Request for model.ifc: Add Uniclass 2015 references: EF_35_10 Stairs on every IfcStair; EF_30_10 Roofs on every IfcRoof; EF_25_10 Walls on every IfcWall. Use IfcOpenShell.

First a look at what the model holds.

```python
import ifcopenshell

model = ifcopenshell.open("model.ifc")
print(model.schema)
print("classifications:", [c.Name for c in model.by_type("IfcClassification")])
for ifc_class in ("IfcDoor", "IfcRoof", "IfcStair", "IfcWall", "IfcWindow"):
    print(ifc_class, len(model.by_type(ifc_class)))
```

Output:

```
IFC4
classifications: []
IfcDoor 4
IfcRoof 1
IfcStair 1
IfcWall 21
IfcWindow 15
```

```python
import ifcopenshell
import ifcopenshell.api.classification

model = ifcopenshell.open("model.ifc")

system = ifcopenshell.api.classification.add_classification(model, classification="Uniclass 2015")

codes = {
    "IfcStair": ("EF_35_10", "Stairs"),
    "IfcRoof": ("EF_30_10", "Roofs"),
    "IfcWall": ("EF_25_10", "Walls"),
}
for ifc_class, (code, name) in codes.items():
    products = model.by_type(ifc_class)
    ifcopenshell.api.classification.add_reference(
        model, products=products, classification=system, identification=code, name=name
    )
    print(code, len(products))

model.write("model_v2.ifc")
```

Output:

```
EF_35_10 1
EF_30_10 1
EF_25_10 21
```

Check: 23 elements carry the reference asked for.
